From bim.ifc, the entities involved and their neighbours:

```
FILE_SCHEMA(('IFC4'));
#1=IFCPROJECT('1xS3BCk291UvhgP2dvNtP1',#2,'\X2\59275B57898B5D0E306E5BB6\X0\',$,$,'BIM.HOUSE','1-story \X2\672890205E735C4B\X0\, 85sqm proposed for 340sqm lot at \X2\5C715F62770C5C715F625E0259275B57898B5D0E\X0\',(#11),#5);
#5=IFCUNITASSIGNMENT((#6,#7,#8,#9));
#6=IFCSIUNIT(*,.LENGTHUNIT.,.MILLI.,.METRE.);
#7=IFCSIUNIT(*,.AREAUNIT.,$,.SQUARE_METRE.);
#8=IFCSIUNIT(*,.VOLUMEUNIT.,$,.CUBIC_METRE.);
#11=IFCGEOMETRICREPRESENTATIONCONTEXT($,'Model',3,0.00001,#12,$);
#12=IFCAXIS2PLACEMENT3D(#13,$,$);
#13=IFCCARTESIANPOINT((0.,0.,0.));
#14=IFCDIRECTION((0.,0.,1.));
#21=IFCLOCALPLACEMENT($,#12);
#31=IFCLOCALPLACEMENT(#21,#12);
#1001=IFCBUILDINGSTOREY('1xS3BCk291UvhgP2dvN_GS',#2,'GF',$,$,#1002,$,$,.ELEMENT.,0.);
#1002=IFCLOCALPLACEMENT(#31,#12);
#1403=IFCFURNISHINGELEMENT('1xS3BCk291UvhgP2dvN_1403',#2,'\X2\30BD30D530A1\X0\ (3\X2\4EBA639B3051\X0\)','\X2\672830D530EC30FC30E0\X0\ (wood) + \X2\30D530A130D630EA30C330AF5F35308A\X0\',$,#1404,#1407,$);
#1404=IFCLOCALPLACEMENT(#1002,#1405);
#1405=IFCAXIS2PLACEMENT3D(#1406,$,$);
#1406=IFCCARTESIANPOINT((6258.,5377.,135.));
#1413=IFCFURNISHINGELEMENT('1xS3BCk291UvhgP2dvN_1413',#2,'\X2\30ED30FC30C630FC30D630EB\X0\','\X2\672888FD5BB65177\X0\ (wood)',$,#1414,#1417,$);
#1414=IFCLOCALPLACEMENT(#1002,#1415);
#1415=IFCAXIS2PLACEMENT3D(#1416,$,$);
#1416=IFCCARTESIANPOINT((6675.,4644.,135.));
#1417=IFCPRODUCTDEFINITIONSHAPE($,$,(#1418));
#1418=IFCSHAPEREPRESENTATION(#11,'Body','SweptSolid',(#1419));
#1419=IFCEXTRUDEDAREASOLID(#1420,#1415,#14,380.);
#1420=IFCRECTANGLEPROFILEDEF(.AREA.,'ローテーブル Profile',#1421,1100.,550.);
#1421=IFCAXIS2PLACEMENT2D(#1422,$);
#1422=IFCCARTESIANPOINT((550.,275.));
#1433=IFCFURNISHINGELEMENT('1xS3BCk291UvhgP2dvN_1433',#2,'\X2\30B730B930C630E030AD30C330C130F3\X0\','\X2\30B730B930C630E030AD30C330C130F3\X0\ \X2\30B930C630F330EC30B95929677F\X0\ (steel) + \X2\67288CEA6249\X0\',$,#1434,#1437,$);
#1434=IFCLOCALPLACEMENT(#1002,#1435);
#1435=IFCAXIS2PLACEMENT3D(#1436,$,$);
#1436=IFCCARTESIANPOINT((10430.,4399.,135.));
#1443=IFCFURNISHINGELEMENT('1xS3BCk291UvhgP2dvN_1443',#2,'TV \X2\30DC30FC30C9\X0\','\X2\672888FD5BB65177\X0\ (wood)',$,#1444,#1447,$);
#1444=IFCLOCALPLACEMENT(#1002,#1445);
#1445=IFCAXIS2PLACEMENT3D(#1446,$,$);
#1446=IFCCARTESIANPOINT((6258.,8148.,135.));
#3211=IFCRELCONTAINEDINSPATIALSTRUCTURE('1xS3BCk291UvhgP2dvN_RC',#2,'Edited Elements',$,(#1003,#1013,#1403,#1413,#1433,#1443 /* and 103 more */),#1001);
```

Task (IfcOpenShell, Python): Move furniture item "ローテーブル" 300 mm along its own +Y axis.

```python
import ifcopenshell
import ifcopenshell.api.geometry
import ifcopenshell.util.placement
import ifcopenshell.util.unit

model = ifcopenshell.open("bim.ifc")
unit_scale = ifcopenshell.util.unit.calculate_unit_scale(model)

item = model.by_id(1413)
matrix = ifcopenshell.util.placement.get_local_placement(item.ObjectPlacement)
matrix[:3, 3] += matrix[:3, 1] * 0.3 / unit_scale
ifcopenshell.api.geometry.edit_object_placement(model, product=item, matrix=matrix, is_si=False)

print(ifcopenshell.util.placement.get_local_placement(item.ObjectPlacement).round(3) + 0.0)

model.write("bim_rev.ifc")
```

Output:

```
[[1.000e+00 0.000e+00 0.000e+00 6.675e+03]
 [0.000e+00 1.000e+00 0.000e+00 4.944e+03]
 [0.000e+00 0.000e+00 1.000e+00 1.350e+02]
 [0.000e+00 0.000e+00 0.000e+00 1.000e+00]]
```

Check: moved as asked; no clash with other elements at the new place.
